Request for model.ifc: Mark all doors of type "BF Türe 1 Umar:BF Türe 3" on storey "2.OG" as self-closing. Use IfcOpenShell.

First a look at what the model holds.

```python
import ifcopenshell
import ifcopenshell.util.element

model = ifcopenshell.open("model.ifc")
print(model.schema)
storey = next(s for s in model.by_type("IfcBuildingStorey") if s.Name == "2.OG")
doors = [e for e in ifcopenshell.util.element.get_decomposition(storey) if e.is_a("IfcDoor")]
seen = {}
for e in doors:
    element_type = ifcopenshell.util.element.get_type(e)
    key = (element_type.Name if element_type != e and element_type else None, ifcopenshell.util.element.get_pset(e, "Pset_DoorCommon", "SelfClosing"))
    seen[key] = seen.get(key, 0) + 1
for (name, value), count in sorted(seen.items(), key=str):
    print(count, "x", name, "|", value)
```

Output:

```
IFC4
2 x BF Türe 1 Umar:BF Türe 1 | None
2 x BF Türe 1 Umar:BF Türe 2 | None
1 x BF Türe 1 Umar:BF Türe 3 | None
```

```python
import ifcopenshell
import ifcopenshell.api.pset
import ifcopenshell.util.element

model = ifcopenshell.open("model.ifc")

storey = next(s for s in model.by_type("IfcBuildingStorey") if s.Name == "2.OG")
doors = [e for e in ifcopenshell.util.element.get_decomposition(storey) if e.is_a("IfcDoor")]

count = 0
for e in doors:
    element_type = ifcopenshell.util.element.get_type(e)
    if element_type in (None, e) or element_type.Name != "BF Türe 1 Umar:BF Türe 3":
        continue
    # add_pset returns the element's existing set when there is one.
    pset = ifcopenshell.api.pset.add_pset(model, product=e, name="Pset_DoorCommon")
    ifcopenshell.api.pset.edit_pset(model, pset=pset, properties={"SelfClosing": True})
    count += 1

print(count, "doors updated")

model.write("model_v2.ifc")
```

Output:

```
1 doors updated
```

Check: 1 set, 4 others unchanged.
